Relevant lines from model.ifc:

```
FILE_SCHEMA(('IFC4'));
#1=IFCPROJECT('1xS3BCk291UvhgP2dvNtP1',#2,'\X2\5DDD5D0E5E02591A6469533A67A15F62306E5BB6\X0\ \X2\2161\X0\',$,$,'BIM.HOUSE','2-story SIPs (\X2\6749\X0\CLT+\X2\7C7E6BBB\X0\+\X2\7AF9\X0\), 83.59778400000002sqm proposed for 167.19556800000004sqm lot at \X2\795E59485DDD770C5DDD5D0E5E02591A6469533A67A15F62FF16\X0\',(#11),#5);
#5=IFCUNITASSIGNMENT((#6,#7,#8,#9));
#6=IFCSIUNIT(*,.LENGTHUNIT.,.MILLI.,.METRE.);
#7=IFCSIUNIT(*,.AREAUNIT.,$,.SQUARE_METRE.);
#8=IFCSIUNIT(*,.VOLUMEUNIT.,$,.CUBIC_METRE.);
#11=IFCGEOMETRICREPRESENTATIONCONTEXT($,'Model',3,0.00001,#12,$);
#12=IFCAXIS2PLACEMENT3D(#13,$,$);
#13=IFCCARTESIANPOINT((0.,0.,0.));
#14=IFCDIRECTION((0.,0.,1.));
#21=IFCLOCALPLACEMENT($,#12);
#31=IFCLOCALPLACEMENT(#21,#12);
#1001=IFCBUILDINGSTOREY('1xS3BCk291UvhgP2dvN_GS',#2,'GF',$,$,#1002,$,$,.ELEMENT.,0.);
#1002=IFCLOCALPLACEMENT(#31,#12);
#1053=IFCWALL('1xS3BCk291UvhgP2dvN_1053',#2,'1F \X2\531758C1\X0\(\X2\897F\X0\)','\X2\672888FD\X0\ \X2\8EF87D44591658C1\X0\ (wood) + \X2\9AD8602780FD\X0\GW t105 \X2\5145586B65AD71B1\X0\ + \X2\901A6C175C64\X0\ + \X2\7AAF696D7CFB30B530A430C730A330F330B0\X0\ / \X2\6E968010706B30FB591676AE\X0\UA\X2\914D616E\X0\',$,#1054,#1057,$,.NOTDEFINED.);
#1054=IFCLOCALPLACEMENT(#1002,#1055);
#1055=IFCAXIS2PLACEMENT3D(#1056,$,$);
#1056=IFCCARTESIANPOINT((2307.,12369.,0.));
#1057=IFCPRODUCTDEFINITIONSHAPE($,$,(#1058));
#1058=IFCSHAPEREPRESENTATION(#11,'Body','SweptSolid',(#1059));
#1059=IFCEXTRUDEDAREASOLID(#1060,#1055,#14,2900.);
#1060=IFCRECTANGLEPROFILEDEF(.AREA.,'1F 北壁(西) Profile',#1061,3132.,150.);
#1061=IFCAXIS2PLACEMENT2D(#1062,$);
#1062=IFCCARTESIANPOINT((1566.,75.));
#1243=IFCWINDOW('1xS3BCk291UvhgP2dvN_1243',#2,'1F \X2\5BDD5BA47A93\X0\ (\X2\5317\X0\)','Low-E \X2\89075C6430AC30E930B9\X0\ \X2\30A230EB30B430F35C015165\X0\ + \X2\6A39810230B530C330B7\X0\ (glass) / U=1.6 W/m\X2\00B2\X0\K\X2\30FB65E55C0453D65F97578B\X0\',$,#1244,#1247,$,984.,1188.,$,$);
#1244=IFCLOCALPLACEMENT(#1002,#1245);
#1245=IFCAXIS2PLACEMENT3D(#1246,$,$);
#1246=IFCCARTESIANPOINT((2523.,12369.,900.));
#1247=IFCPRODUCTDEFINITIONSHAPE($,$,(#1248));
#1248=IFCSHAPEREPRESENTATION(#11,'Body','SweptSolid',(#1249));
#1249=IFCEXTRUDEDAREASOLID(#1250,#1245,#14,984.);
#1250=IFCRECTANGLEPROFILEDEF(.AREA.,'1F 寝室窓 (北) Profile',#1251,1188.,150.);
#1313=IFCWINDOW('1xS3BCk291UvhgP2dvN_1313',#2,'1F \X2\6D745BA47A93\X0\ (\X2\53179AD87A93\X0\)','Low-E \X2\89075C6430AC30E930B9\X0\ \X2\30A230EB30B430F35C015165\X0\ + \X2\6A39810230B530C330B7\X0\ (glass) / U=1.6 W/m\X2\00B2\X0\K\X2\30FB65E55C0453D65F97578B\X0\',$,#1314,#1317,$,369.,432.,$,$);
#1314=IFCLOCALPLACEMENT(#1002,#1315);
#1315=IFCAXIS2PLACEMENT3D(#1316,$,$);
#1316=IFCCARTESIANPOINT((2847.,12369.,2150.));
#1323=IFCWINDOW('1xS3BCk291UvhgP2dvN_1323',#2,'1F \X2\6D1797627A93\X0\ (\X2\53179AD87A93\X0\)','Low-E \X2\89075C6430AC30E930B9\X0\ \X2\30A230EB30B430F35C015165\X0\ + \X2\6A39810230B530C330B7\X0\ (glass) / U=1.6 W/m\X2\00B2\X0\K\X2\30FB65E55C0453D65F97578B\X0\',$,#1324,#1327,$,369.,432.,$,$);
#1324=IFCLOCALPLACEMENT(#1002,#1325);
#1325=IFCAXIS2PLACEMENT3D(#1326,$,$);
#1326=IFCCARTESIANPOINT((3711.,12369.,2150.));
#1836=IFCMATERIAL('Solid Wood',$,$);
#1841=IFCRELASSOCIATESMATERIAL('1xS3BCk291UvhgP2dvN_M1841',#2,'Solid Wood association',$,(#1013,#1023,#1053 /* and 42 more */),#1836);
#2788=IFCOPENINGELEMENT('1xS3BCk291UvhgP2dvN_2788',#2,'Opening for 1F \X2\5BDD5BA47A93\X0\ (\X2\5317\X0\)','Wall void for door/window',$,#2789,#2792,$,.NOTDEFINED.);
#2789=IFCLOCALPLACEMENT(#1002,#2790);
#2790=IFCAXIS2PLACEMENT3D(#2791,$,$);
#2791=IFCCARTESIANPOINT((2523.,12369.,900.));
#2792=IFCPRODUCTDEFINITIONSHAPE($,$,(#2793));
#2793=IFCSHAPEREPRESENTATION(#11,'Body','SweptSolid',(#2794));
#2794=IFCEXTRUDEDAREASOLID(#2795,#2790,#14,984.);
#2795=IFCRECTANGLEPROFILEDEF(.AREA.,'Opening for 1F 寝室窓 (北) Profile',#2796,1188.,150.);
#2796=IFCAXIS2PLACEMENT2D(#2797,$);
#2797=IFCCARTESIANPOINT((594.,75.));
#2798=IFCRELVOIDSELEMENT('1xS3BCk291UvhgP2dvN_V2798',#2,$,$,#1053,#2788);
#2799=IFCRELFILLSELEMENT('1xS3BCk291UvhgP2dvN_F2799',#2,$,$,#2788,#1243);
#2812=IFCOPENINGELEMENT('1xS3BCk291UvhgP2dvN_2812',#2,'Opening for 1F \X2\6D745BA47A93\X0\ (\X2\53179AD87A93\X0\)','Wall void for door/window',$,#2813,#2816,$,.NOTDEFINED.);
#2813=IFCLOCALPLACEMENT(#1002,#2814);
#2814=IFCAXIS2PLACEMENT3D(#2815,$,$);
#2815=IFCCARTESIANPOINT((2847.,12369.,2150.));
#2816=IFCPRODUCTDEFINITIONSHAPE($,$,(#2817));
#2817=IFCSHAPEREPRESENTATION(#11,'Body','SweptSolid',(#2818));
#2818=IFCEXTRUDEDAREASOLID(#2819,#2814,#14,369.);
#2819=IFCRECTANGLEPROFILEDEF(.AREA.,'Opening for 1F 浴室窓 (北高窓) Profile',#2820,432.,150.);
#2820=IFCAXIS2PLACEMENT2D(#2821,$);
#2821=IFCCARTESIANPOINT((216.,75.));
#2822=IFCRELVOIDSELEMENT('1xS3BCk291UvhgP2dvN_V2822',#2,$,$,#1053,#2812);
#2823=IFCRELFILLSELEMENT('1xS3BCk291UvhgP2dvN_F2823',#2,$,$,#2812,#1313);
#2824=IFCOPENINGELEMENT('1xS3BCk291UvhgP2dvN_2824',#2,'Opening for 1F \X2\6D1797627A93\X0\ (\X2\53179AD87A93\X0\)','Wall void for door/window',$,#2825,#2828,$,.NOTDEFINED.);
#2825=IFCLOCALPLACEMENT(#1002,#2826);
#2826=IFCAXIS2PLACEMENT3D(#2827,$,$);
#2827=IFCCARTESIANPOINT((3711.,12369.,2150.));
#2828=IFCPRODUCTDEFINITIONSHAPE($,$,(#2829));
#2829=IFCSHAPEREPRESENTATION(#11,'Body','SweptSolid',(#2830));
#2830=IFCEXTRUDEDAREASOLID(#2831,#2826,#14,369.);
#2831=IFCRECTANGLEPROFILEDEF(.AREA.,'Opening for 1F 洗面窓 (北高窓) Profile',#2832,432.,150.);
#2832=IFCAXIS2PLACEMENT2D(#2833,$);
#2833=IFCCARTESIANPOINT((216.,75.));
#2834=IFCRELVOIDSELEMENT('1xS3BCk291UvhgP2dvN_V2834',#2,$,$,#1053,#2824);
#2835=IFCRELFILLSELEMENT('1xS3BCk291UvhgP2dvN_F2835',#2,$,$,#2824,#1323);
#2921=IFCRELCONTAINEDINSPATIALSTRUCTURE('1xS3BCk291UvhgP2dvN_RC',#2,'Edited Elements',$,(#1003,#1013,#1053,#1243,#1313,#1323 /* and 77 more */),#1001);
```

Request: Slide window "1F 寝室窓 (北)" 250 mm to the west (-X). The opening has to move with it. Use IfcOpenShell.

```python
import ifcopenshell
import ifcopenshell.api.geometry
import ifcopenshell.util.placement

model = ifcopenshell.open("model.ifc")

window = model.by_guid("1xS3BCk291UvhgP2dvN_1243")
opening = window.FillsVoids[0].RelatingOpeningElement
wall = opening.VoidsElements[0].RelatingBuildingElement

wall_matrix = ifcopenshell.util.placement.get_local_placement(wall.ObjectPlacement)
shift = wall_matrix[:3, 0] * -250.0
before = ifcopenshell.util.placement.get_local_placement(window.ObjectPlacement)[:3, 3].copy()

# The window is not placed relative to its opening, so move both.
for product in (opening, window):
    matrix = ifcopenshell.util.placement.get_local_placement(product.ObjectPlacement)
    matrix[:3, 3] += shift
    ifcopenshell.api.geometry.edit_object_placement(model, product=product, matrix=matrix, is_si=False)

after = ifcopenshell.util.placement.get_local_placement(window.ObjectPlacement)[:3, 3]
print("window moved by", (after - before).round(3) + 0.0)

model.write("model_v2.ifc")
```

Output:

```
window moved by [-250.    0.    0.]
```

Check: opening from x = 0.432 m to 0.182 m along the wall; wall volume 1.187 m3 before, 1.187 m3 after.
